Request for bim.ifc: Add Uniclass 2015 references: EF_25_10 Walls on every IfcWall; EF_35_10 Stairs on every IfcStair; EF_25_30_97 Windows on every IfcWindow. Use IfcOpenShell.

First a look at what the model holds.

```python
import ifcopenshell

model = ifcopenshell.open("bim.ifc")
print(model.schema)
print("classifications:", [c.Name for c in model.by_type("IfcClassification")])
for ifc_class in ("IfcDoor", "IfcRoof", "IfcStair", "IfcWall", "IfcWindow"):
    print(ifc_class, len(model.by_type(ifc_class)))
```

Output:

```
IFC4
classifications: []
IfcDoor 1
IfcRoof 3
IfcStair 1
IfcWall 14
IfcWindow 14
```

```python
import ifcopenshell
import ifcopenshell.api.classification

model = ifcopenshell.open("bim.ifc")

system = ifcopenshell.api.classification.add_classification(model, classification="Uniclass 2015")

codes = {
    "IfcWall": ("EF_25_10", "Walls"),
    "IfcStair": ("EF_35_10", "Stairs"),
    "IfcWindow": ("EF_25_30_97", "Windows"),
}
for ifc_class, (code, name) in codes.items():
    products = model.by_type(ifc_class)
    ifcopenshell.api.classification.add_reference(
        model, products=products, classification=system, identification=code, name=name
    )
    print(code, len(products))

model.write("bim_rev.ifc")
```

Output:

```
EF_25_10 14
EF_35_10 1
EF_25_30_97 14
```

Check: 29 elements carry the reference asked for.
